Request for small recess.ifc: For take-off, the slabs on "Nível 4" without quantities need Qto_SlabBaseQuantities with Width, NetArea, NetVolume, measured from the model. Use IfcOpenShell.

First a look at what the model holds.

```python
import ifcopenshell
import ifcopenshell.util.element
import ifcopenshell.util.unit

model = ifcopenshell.open("small recess.ifc")
print(model.schema)
for unit_type in ("LENGTHUNIT", "AREAUNIT", "VOLUMEUNIT"):
    print(unit_type, ifcopenshell.util.unit.calculate_unit_scale(model, unit_type))
storey = next(s for s in model.by_type("IfcBuildingStorey") if s.Name == "Nível 4")
slabs = [e for e in ifcopenshell.util.element.get_decomposition(storey) if e.is_a("IfcSlab")]
for e in sorted(slabs, key=lambda e: e.id()):
    print(e.id(), e.is_a(), e.Name, list(ifcopenshell.util.element.get_psets(e, qtos_only=True)), sep=" | ")
```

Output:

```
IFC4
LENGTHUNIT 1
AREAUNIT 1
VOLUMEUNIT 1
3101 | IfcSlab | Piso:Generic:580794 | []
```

```python
import ifcopenshell
import ifcopenshell.api.pset
import ifcopenshell.geom
import ifcopenshell.util.element
import ifcopenshell.util.shape
import ifcopenshell.util.unit

model = ifcopenshell.open("small recess.ifc")
unit_scale = ifcopenshell.util.unit.calculate_unit_scale(model)
area_scale = ifcopenshell.util.unit.calculate_unit_scale(model, "AREAUNIT")
volume_scale = ifcopenshell.util.unit.calculate_unit_scale(model, "VOLUMEUNIT")
settings = ifcopenshell.geom.settings()

storey = next(s for s in model.by_type("IfcBuildingStorey") if s.Name == "Nível 4")
slabs = [e for e in ifcopenshell.util.element.get_decomposition(storey) if e.is_a("IfcSlab")]

for e in sorted(slabs, key=lambda e: e.id()):
    if ifcopenshell.util.element.get_psets(e, qtos_only=True, should_inherit=False):
        continue
    # Geometry comes back in metres, in the element's own axes.
    shape = ifcopenshell.geom.create_shape(settings, e)
    values = {
        "Width": ifcopenshell.util.shape.get_z(shape.geometry) / unit_scale,
        "NetArea": ifcopenshell.util.shape.get_footprint_area(shape.geometry) / area_scale,
        "NetVolume": ifcopenshell.util.shape.get_volume(shape.geometry) / volume_scale,
    }
    qto = ifcopenshell.api.pset.add_qto(model, product=e, name="Qto_SlabBaseQuantities")
    ifcopenshell.api.pset.edit_qto(model, qto=qto, properties=values)
    print(e.id(), {k: round(v, 3) for k, v in values.items()})

model.write("small recess_v2.ifc")
```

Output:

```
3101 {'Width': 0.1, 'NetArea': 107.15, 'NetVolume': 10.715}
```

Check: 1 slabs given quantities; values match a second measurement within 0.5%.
